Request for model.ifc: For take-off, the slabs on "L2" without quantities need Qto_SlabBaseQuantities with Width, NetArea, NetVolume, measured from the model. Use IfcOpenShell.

First a look at what the model holds.

```python
import ifcopenshell
import ifcopenshell.util.element
import ifcopenshell.util.unit

model = ifcopenshell.open("model.ifc")
print(model.schema)
for unit_type in ("LENGTHUNIT", "AREAUNIT", "VOLUMEUNIT"):
    print(unit_type, ifcopenshell.util.unit.calculate_unit_scale(model, unit_type))
storey = next(s for s in model.by_type("IfcBuildingStorey") if s.Name == "L2")
slabs = [e for e in ifcopenshell.util.element.get_decomposition(storey) if e.is_a("IfcSlab")]
for e in sorted(slabs, key=lambda e: e.id()):
    print(e.id(), e.is_a(), e.Name, list(ifcopenshell.util.element.get_psets(e, qtos_only=True)), sep=" | ")
```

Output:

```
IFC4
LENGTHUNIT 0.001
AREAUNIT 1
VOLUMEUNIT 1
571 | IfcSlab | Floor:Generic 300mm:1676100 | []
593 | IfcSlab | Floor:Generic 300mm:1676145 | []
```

```python
import ifcopenshell
import ifcopenshell.api.pset
import ifcopenshell.geom
import ifcopenshell.util.element
import ifcopenshell.util.shape
import ifcopenshell.util.unit

model = ifcopenshell.open("model.ifc")
unit_scale = ifcopenshell.util.unit.calculate_unit_scale(model)
area_scale = ifcopenshell.util.unit.calculate_unit_scale(model, "AREAUNIT")
volume_scale = ifcopenshell.util.unit.calculate_unit_scale(model, "VOLUMEUNIT")
settings = ifcopenshell.geom.settings()

storey = next(s for s in model.by_type("IfcBuildingStorey") if s.Name == "L2")
slabs = [e for e in ifcopenshell.util.element.get_decomposition(storey) if e.is_a("IfcSlab")]

for e in sorted(slabs, key=lambda e: e.id()):
    if ifcopenshell.util.element.get_psets(e, qtos_only=True, should_inherit=False):
        continue
    # Geometry comes back in metres, in the element's own axes.
    shape = ifcopenshell.geom.create_shape(settings, e)
    values = {
        "Width": ifcopenshell.util.shape.get_z(shape.geometry) / unit_scale,
        "NetArea": ifcopenshell.util.shape.get_footprint_area(shape.geometry) / area_scale,
        "NetVolume": ifcopenshell.util.shape.get_volume(shape.geometry) / volume_scale,
    }
    qto = ifcopenshell.api.pset.add_qto(model, product=e, name="Qto_SlabBaseQuantities")
    ifcopenshell.api.pset.edit_qto(model, qto=qto, properties=values)
    print(e.id(), {k: round(v, 3) for k, v in values.items()})

model.write("model-out.ifc")
```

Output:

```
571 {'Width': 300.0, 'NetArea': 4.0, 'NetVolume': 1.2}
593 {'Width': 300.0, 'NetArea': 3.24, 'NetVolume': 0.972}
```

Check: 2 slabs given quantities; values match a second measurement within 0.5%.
